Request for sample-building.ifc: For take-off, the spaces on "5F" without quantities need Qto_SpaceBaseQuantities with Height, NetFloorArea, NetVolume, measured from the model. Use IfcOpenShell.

First a look at what the model holds.

```python
import ifcopenshell
import ifcopenshell.util.element
import ifcopenshell.util.unit

model = ifcopenshell.open("sample-building.ifc")
print(model.schema)
for unit_type in ("LENGTHUNIT", "AREAUNIT", "VOLUMEUNIT"):
    print(unit_type, ifcopenshell.util.unit.calculate_unit_scale(model, unit_type))
storey = next(s for s in model.by_type("IfcBuildingStorey") if s.Name == "5F")
spaces = [e for e in ifcopenshell.util.element.get_decomposition(storey) if e.is_a("IfcSpace")]
for e in sorted(spaces, key=lambda e: e.id()):
    print(e.id(), e.is_a(), e.Name, list(ifcopenshell.util.element.get_psets(e, qtos_only=True)), sep=" | ")
```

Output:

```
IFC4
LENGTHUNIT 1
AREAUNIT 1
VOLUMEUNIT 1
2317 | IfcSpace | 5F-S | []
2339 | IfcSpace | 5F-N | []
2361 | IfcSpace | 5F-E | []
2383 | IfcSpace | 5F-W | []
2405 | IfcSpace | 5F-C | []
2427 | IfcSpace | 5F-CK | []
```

```python
import ifcopenshell
import ifcopenshell.api.pset
import ifcopenshell.geom
import ifcopenshell.util.element
import ifcopenshell.util.shape
import ifcopenshell.util.unit

model = ifcopenshell.open("sample-building.ifc")
unit_scale = ifcopenshell.util.unit.calculate_unit_scale(model)
area_scale = ifcopenshell.util.unit.calculate_unit_scale(model, "AREAUNIT")
volume_scale = ifcopenshell.util.unit.calculate_unit_scale(model, "VOLUMEUNIT")
settings = ifcopenshell.geom.settings()

storey = next(s for s in model.by_type("IfcBuildingStorey") if s.Name == "5F")
spaces = [e for e in ifcopenshell.util.element.get_decomposition(storey) if e.is_a("IfcSpace")]

for e in sorted(spaces, key=lambda e: e.id()):
    if ifcopenshell.util.element.get_psets(e, qtos_only=True, should_inherit=False):
        continue
    # Geometry comes back in metres, in the element's own axes.
    shape = ifcopenshell.geom.create_shape(settings, e)
    values = {
        "Height": ifcopenshell.util.shape.get_z(shape.geometry) / unit_scale,
        "NetFloorArea": ifcopenshell.util.shape.get_footprint_area(shape.geometry) / area_scale,
        "NetVolume": ifcopenshell.util.shape.get_volume(shape.geometry) / volume_scale,
    }
    qto = ifcopenshell.api.pset.add_qto(model, product=e, name="Qto_SpaceBaseQuantities")
    ifcopenshell.api.pset.edit_qto(model, qto=qto, properties=values)
    print(e.id(), {k: round(v, 3) for k, v in values.items()})

model.write("sample-building_rev.ifc")
```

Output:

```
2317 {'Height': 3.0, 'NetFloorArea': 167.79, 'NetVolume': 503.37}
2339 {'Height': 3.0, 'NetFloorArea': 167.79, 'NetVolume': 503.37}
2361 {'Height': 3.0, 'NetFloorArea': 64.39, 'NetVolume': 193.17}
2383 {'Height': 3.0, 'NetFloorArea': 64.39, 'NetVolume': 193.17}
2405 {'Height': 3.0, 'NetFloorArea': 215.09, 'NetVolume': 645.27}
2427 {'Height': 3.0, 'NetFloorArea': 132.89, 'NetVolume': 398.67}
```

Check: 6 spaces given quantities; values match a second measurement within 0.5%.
